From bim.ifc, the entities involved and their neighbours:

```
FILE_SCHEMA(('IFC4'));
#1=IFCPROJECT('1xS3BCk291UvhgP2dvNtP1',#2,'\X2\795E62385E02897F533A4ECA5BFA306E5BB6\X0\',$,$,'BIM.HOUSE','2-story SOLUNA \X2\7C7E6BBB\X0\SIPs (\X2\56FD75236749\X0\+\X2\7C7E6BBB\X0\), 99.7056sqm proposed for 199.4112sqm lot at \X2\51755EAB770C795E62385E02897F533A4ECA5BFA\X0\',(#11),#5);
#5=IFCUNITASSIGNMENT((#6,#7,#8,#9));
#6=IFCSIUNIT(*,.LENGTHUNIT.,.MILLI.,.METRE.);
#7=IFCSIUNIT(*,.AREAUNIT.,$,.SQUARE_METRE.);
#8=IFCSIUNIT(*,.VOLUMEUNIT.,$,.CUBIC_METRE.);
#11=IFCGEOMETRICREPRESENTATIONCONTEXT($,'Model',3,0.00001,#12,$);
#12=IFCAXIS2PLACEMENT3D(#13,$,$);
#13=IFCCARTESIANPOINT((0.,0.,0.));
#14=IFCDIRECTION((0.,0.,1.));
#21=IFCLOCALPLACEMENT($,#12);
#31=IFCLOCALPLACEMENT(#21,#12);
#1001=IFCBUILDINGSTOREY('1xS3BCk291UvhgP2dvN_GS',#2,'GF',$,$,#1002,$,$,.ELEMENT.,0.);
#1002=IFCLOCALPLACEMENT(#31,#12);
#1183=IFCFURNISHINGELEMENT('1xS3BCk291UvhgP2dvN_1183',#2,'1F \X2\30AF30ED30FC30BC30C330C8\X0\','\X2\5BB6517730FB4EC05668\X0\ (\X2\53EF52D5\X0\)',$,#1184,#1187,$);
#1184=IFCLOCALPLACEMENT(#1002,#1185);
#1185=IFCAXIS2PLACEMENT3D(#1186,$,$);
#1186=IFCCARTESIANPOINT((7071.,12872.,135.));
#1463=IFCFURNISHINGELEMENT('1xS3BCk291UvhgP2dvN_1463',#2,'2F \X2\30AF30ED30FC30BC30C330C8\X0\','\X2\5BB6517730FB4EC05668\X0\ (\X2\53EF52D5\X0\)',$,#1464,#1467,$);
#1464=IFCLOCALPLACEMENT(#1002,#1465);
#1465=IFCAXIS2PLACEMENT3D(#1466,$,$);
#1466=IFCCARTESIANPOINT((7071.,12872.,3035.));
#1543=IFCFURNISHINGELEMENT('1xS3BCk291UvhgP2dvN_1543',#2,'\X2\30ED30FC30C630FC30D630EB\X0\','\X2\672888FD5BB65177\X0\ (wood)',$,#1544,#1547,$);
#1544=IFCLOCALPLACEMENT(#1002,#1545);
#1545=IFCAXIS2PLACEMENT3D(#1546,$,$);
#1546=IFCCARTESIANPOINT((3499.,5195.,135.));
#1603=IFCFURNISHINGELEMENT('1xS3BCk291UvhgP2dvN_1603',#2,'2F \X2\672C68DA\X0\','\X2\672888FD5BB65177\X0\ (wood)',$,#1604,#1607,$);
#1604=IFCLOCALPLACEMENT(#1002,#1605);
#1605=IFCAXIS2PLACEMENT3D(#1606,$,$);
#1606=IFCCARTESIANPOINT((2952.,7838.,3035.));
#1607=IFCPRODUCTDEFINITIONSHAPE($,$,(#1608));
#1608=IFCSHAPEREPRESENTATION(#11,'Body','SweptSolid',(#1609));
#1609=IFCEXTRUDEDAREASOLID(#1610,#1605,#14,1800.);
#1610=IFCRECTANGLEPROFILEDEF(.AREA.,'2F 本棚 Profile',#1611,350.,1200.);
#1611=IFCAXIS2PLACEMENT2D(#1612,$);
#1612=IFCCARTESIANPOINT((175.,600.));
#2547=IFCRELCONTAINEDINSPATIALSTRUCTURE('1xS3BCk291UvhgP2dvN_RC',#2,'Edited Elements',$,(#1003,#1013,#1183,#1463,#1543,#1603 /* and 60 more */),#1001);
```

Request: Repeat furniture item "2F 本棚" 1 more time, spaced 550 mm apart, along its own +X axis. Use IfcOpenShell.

```python
import ifcopenshell
import ifcopenshell.api.geometry
import ifcopenshell.api.root
import ifcopenshell.util.element
import ifcopenshell.util.placement
import ifcopenshell.util.unit

model = ifcopenshell.open("bim.ifc")
unit_scale = ifcopenshell.util.unit.calculate_unit_scale(model)


def reuse_history(source, copy):
    """copy_class also copies each property set's owner history, people and application; keep the originals."""
    for rel in copy.IsDefinedBy:
        if rel.is_a("IfcRelDefinesByProperties") and (history := rel.RelatingPropertyDefinition.OwnerHistory):
            rel.RelatingPropertyDefinition.OwnerHistory = source.OwnerHistory
            ifcopenshell.util.element.remove_deep2(model, history)


source = model.by_guid("1xS3BCk291UvhgP2dvN_1603")
base = ifcopenshell.util.placement.get_local_placement(source.ObjectPlacement)
step = base[:3, 0] * 0.55 / unit_scale

for i in range(1, 2):
    copy = ifcopenshell.api.root.copy_class(model, product=source)
    copy.Representation = ifcopenshell.util.element.copy_deep(
        model, source.Representation, exclude=["IfcGeometricRepresentationContext", "IfcRepresentationMap"]
    )
    reuse_history(source, copy)
    matrix = base.copy()
    matrix[:3, 3] += i * step
    print("added at", matrix[:3, 3].round(3) + 0.0)
    ifcopenshell.api.geometry.edit_object_placement(model, product=copy, matrix=matrix, is_si=False)

model.write("bim_rev.ifc")
```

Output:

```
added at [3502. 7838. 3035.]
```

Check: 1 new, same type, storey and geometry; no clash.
